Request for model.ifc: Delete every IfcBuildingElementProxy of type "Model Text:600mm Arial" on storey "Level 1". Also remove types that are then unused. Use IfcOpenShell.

First a look at what the model holds.

```python
import ifcopenshell
import ifcopenshell.util.element

model = ifcopenshell.open("model.ifc")
print(model.schema)
storey = next(s for s in model.by_type("IfcBuildingStorey") if s.Name == "Level 1")
proxies = [e for e in ifcopenshell.util.element.get_decomposition(storey) if e.is_a("IfcBuildingElementProxy")]
seen = {}
for e in proxies:
    element_type = ifcopenshell.util.element.get_type(e)
    name = element_type.Name if element_type not in (None, e) else None
    seen[name] = seen.get(name, 0) + 1
for name, count in sorted(seen.items(), key=str):
    print(count, "x", name)
```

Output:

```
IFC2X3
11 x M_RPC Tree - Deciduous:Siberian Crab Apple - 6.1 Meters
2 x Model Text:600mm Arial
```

```python
import ifcopenshell
import ifcopenshell.api.root
import ifcopenshell.util.element

model = ifcopenshell.open("model.ifc")

storey = next(s for s in model.by_type("IfcBuildingStorey") if s.Name == "Level 1")
proxies = [e for e in ifcopenshell.util.element.get_decomposition(storey) if e.is_a("IfcBuildingElementProxy")]
targets = [e for e in proxies if (t := ifcopenshell.util.element.get_type(e)) not in (None, e) and t.Name == "Model Text:600mm Arial"]
types = {ifcopenshell.util.element.get_type(e) for e in targets} - {None, *targets}

for e in targets:
    ifcopenshell.api.root.remove_product(model, product=e)
print(len(targets), "removed")

unused = [t for t in types if not ifcopenshell.util.element.get_types(t)]
for t in unused:
    ifcopenshell.api.root.remove_product(model, product=t)
print(len(unused), "unused types removed")

model.write("model-out.ifc")
```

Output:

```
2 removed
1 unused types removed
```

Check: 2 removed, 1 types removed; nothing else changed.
